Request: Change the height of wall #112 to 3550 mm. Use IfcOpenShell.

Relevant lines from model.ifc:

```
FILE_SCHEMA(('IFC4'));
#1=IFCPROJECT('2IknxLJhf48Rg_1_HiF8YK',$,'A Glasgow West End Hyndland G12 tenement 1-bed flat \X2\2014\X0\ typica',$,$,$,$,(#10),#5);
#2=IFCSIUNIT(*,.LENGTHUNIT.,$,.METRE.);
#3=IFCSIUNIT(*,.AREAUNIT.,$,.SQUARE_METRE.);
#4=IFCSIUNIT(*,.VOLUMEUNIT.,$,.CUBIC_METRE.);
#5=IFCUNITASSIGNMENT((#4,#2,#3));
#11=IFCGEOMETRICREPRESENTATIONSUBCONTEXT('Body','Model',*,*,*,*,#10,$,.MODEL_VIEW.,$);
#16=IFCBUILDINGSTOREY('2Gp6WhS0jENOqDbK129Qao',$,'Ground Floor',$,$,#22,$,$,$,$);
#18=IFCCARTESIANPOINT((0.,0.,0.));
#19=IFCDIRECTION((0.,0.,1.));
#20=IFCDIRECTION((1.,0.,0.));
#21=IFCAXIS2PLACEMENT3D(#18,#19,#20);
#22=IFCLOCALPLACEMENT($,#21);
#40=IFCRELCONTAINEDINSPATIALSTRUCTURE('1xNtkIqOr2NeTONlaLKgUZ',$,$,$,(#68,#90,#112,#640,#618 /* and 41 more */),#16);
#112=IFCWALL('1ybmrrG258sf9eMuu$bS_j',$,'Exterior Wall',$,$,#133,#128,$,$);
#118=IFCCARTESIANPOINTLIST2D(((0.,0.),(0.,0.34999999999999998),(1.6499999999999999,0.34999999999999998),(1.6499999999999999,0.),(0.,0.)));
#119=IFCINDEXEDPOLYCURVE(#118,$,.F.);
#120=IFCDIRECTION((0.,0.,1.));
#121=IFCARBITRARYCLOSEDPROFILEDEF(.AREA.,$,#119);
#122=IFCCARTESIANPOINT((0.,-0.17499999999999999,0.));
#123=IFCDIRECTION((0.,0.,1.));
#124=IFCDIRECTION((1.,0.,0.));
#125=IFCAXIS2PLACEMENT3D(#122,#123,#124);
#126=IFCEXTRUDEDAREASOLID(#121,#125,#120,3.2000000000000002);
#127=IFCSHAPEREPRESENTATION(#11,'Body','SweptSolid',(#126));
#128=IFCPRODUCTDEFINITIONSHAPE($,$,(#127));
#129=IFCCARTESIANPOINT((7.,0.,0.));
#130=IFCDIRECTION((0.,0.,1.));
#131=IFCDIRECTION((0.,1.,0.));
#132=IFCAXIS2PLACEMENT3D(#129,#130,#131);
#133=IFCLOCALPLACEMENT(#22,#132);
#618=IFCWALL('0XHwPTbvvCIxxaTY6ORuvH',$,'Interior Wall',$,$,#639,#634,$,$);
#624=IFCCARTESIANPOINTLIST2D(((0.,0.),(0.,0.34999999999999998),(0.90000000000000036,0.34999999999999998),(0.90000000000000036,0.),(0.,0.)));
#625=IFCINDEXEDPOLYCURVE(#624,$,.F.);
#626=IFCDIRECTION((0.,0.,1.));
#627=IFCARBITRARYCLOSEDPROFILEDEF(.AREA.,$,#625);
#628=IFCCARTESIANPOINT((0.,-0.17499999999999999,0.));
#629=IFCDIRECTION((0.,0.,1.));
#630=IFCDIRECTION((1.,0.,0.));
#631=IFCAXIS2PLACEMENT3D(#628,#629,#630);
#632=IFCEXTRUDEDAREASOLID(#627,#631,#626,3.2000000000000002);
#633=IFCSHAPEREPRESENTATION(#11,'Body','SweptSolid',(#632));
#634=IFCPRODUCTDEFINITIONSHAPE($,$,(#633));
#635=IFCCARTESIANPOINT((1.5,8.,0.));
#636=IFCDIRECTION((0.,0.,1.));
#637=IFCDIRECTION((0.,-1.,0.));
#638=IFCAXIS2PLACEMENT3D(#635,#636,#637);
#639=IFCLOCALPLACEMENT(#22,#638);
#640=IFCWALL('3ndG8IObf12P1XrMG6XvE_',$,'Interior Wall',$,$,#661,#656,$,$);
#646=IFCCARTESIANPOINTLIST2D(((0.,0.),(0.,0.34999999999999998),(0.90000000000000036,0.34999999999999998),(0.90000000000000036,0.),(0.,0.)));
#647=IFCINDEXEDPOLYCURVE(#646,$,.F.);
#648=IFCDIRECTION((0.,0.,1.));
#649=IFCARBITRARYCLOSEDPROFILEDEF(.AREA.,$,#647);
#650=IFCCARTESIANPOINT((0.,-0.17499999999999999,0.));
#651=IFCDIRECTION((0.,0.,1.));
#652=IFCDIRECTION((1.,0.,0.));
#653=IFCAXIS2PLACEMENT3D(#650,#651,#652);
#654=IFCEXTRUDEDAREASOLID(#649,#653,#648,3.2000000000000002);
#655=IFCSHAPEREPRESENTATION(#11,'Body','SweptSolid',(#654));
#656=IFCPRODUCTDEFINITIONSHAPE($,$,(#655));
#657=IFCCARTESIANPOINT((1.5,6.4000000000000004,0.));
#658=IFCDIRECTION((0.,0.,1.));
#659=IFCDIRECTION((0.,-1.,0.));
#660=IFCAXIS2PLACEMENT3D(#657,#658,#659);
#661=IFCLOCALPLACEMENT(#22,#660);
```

```python
import ifcopenshell
import ifcopenshell.geom
import ifcopenshell.util.representation
import ifcopenshell.util.shape

model = ifcopenshell.open("model.ifc")
settings = ifcopenshell.geom.settings()


def volume(element):
    """Net volume in cubic metres, openings subtracted."""
    shape = ifcopenshell.geom.create_shape(settings, element)
    return ifcopenshell.util.shape.get_volume(shape.geometry)


wall = model.by_guid("1ybmrrG258sf9eMuu$bS_j")
before = volume(wall)

body = ifcopenshell.util.representation.get_representation(wall, "Model", "Body")
solid = body.Items[0]
old_height = solid.Depth
solid.Depth = 3.55
after = volume(wall)

print(f"height {old_height:g} -> {solid.Depth:g}, volume {before:.3f} -> {after:.3f} m3")

model.write("model_edited.ifc")
```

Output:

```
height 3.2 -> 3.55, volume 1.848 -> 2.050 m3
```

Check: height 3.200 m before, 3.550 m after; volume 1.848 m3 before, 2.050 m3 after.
